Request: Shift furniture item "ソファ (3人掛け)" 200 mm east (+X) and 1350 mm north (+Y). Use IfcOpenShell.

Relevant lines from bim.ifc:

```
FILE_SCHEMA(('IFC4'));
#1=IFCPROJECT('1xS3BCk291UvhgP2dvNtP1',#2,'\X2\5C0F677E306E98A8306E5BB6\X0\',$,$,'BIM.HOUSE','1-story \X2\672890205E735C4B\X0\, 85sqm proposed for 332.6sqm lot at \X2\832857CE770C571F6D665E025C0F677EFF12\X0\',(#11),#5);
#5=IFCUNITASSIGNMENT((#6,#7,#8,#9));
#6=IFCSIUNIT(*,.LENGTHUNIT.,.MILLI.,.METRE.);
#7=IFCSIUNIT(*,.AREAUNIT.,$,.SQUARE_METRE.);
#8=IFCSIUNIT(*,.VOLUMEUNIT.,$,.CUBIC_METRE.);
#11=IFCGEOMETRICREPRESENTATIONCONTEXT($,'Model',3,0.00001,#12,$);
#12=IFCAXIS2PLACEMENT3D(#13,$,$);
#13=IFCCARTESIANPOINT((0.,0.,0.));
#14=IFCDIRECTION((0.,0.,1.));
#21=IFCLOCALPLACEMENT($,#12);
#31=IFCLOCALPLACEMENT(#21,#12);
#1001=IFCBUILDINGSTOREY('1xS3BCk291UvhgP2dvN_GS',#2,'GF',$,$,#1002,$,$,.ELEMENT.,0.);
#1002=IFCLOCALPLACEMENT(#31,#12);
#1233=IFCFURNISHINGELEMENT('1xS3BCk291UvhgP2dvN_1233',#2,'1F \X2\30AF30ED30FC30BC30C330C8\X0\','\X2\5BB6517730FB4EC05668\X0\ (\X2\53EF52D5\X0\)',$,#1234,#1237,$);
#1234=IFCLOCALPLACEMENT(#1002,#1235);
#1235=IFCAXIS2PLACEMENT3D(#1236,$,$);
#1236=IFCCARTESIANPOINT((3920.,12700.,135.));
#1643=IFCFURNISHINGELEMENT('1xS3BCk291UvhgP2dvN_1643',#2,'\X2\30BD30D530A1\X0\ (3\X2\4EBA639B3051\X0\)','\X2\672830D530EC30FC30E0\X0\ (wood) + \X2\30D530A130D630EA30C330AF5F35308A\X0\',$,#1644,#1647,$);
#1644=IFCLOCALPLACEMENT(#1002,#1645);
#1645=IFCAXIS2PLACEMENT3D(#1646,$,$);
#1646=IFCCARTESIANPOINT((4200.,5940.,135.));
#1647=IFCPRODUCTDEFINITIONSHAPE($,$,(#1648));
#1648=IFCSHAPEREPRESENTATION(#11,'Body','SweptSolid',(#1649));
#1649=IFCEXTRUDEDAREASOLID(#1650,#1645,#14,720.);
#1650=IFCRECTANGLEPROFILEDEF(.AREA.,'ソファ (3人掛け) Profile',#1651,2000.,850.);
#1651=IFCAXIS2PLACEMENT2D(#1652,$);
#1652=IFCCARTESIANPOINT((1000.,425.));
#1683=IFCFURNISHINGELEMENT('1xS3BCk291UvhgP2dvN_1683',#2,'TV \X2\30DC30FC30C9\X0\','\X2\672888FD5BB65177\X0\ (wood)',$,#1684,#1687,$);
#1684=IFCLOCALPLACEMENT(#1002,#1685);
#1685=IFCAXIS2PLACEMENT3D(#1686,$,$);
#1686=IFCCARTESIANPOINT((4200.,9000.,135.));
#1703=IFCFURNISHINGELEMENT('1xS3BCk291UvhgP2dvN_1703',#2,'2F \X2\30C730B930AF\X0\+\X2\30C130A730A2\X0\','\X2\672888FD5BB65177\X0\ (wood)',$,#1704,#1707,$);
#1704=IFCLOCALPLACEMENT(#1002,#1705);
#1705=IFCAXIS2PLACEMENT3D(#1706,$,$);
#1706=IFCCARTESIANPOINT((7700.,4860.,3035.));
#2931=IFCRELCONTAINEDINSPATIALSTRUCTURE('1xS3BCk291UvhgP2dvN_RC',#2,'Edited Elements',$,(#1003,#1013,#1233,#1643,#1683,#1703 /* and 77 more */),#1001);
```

```python
import ifcopenshell
import ifcopenshell.api.geometry
import ifcopenshell.util.placement
import ifcopenshell.util.unit

model = ifcopenshell.open("bim.ifc")
unit_scale = ifcopenshell.util.unit.calculate_unit_scale(model)

item = model.by_guid("1xS3BCk291UvhgP2dvN_1643")
matrix = ifcopenshell.util.placement.get_local_placement(item.ObjectPlacement)
matrix[0, 3] += 0.2 / unit_scale
matrix[1, 3] += 1.35 / unit_scale
ifcopenshell.api.geometry.edit_object_placement(model, product=item, matrix=matrix, is_si=False)

print(ifcopenshell.util.placement.get_local_placement(item.ObjectPlacement).round(3) + 0.0)

model.write("bim-out.ifc")
```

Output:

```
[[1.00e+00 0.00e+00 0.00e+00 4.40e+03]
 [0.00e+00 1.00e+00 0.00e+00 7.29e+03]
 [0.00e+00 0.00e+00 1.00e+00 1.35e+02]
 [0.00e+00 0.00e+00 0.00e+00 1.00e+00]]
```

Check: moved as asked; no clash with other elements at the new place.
